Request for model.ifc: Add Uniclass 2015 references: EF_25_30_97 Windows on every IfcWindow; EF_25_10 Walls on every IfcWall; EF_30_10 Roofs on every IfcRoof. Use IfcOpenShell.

First a look at what the model holds.

```python
import ifcopenshell

model = ifcopenshell.open("model.ifc")
print(model.schema)
print("classifications:", [c.Name for c in model.by_type("IfcClassification")])
for ifc_class in ("IfcDoor", "IfcRoof", "IfcStair", "IfcWall", "IfcWindow"):
    print(ifc_class, len(model.by_type(ifc_class)))
```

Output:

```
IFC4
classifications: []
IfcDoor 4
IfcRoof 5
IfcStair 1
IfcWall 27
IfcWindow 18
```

```python
import ifcopenshell
import ifcopenshell.api.classification

model = ifcopenshell.open("model.ifc")

system = ifcopenshell.api.classification.add_classification(model, classification="Uniclass 2015")

codes = {
    "IfcWindow": ("EF_25_30_97", "Windows"),
    "IfcWall": ("EF_25_10", "Walls"),
    "IfcRoof": ("EF_30_10", "Roofs"),
}
for ifc_class, (code, name) in codes.items():
    products = model.by_type(ifc_class)
    ifcopenshell.api.classification.add_reference(
        model, products=products, classification=system, identification=code, name=name
    )
    print(code, len(products))

model.write("model_v2.ifc")
```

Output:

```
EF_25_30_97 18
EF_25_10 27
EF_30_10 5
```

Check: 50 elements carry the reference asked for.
